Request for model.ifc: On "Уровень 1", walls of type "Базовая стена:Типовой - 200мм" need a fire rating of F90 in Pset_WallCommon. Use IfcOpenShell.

First a look at what the model holds.

```python
import ifcopenshell
import ifcopenshell.util.element

model = ifcopenshell.open("model.ifc")
print(model.schema)
storey = next(s for s in model.by_type("IfcBuildingStorey") if s.Name == "Уровень 1")
walls = [e for e in ifcopenshell.util.element.get_decomposition(storey) if e.is_a("IfcWall")]
seen = {}
for e in walls:
    element_type = ifcopenshell.util.element.get_type(e)
    key = (element_type.Name if element_type != e and element_type else None, ifcopenshell.util.element.get_pset(e, "Pset_WallCommon", "FireRating"))
    seen[key] = seen.get(key, 0) + 1
for (name, value), count in sorted(seen.items(), key=str):
    print(count, "x", name, "|", value)
```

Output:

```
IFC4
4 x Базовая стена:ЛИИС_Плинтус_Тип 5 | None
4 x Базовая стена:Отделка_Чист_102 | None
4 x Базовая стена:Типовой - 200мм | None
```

```python
import ifcopenshell
import ifcopenshell.api.pset
import ifcopenshell.util.element

model = ifcopenshell.open("model.ifc")

storey = next(s for s in model.by_type("IfcBuildingStorey") if s.Name == "Уровень 1")
walls = [e for e in ifcopenshell.util.element.get_decomposition(storey) if e.is_a("IfcWall")]

count = 0
for e in walls:
    element_type = ifcopenshell.util.element.get_type(e)
    if element_type in (None, e) or element_type.Name != "Базовая стена:Типовой - 200мм":
        continue
    # add_pset returns the element's existing set when there is one.
    pset = ifcopenshell.api.pset.add_pset(model, product=e, name="Pset_WallCommon")
    ifcopenshell.api.pset.edit_pset(model, pset=pset, properties={"FireRating": "F90"})
    count += 1

print(count, "walls updated")

model.write("model_updated.ifc")
```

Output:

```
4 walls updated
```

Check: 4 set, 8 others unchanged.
